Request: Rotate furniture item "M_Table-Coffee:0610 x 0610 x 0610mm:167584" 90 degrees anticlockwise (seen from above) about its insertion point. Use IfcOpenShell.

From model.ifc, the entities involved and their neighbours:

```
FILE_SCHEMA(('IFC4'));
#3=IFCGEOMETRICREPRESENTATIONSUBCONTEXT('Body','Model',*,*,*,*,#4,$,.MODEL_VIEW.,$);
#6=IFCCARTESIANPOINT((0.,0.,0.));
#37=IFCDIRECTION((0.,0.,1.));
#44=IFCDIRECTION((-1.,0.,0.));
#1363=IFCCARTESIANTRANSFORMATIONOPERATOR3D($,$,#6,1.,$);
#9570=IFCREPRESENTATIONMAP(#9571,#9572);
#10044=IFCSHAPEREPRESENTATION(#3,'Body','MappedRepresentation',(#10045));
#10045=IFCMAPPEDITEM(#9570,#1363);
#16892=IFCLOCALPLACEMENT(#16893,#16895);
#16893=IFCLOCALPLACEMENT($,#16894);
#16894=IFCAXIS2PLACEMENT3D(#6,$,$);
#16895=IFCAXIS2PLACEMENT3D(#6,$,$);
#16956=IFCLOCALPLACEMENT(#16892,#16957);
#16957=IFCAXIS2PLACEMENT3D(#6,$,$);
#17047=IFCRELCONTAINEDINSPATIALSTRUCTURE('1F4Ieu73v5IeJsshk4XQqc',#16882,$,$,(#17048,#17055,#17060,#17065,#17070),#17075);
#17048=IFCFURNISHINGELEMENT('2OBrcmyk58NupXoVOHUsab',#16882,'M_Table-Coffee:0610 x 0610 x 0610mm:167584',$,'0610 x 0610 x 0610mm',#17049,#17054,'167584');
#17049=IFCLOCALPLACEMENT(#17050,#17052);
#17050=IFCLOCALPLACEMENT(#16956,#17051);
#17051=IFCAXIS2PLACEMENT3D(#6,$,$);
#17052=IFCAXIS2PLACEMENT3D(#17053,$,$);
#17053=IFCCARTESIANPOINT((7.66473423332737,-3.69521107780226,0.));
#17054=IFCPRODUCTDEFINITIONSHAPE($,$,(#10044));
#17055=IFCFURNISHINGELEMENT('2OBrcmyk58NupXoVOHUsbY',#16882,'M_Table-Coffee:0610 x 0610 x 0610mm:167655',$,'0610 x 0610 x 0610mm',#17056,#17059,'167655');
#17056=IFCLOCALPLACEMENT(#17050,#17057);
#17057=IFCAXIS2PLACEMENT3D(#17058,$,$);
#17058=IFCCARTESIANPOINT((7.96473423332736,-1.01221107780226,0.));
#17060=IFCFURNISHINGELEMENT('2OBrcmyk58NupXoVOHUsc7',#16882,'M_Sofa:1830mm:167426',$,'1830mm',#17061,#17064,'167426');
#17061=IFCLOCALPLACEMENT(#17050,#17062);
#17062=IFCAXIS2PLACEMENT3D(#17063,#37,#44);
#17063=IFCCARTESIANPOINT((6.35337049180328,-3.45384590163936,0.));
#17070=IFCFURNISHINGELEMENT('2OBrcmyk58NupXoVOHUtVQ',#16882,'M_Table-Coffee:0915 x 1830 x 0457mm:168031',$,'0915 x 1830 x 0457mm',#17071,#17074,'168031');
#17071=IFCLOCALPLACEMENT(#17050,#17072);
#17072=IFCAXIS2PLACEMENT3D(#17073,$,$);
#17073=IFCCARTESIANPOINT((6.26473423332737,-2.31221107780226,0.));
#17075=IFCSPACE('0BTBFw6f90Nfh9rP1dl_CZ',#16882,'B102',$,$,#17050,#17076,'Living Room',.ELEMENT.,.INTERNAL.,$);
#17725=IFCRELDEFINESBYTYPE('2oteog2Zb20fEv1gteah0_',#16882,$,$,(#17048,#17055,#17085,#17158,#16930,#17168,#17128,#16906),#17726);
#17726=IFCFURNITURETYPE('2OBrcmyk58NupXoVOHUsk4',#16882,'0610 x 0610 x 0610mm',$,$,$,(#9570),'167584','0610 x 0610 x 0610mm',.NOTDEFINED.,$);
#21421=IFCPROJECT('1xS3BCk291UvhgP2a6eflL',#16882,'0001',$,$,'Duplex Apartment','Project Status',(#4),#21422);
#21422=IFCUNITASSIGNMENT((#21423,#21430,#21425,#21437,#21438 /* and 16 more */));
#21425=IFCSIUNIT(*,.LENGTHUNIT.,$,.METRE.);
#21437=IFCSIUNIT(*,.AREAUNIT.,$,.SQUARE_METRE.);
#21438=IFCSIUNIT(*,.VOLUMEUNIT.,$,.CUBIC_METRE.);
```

```python
import ifcopenshell
import ifcopenshell.api.geometry
import ifcopenshell.util.placement

model = ifcopenshell.open("model.ifc")

item = model.by_guid("2OBrcmyk58NupXoVOHUsab")
matrix = ifcopenshell.util.placement.get_local_placement(item.ObjectPlacement)
matrix = matrix @ ifcopenshell.util.placement.rotation(90, "Z")
ifcopenshell.api.geometry.edit_object_placement(model, product=item, matrix=matrix, is_si=False)

print(ifcopenshell.util.placement.get_local_placement(item.ObjectPlacement).round(3) + 0.0)

model.write("model-out.ifc")
```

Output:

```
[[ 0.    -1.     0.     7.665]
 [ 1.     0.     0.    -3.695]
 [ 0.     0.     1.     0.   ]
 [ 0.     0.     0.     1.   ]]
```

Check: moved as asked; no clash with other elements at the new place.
